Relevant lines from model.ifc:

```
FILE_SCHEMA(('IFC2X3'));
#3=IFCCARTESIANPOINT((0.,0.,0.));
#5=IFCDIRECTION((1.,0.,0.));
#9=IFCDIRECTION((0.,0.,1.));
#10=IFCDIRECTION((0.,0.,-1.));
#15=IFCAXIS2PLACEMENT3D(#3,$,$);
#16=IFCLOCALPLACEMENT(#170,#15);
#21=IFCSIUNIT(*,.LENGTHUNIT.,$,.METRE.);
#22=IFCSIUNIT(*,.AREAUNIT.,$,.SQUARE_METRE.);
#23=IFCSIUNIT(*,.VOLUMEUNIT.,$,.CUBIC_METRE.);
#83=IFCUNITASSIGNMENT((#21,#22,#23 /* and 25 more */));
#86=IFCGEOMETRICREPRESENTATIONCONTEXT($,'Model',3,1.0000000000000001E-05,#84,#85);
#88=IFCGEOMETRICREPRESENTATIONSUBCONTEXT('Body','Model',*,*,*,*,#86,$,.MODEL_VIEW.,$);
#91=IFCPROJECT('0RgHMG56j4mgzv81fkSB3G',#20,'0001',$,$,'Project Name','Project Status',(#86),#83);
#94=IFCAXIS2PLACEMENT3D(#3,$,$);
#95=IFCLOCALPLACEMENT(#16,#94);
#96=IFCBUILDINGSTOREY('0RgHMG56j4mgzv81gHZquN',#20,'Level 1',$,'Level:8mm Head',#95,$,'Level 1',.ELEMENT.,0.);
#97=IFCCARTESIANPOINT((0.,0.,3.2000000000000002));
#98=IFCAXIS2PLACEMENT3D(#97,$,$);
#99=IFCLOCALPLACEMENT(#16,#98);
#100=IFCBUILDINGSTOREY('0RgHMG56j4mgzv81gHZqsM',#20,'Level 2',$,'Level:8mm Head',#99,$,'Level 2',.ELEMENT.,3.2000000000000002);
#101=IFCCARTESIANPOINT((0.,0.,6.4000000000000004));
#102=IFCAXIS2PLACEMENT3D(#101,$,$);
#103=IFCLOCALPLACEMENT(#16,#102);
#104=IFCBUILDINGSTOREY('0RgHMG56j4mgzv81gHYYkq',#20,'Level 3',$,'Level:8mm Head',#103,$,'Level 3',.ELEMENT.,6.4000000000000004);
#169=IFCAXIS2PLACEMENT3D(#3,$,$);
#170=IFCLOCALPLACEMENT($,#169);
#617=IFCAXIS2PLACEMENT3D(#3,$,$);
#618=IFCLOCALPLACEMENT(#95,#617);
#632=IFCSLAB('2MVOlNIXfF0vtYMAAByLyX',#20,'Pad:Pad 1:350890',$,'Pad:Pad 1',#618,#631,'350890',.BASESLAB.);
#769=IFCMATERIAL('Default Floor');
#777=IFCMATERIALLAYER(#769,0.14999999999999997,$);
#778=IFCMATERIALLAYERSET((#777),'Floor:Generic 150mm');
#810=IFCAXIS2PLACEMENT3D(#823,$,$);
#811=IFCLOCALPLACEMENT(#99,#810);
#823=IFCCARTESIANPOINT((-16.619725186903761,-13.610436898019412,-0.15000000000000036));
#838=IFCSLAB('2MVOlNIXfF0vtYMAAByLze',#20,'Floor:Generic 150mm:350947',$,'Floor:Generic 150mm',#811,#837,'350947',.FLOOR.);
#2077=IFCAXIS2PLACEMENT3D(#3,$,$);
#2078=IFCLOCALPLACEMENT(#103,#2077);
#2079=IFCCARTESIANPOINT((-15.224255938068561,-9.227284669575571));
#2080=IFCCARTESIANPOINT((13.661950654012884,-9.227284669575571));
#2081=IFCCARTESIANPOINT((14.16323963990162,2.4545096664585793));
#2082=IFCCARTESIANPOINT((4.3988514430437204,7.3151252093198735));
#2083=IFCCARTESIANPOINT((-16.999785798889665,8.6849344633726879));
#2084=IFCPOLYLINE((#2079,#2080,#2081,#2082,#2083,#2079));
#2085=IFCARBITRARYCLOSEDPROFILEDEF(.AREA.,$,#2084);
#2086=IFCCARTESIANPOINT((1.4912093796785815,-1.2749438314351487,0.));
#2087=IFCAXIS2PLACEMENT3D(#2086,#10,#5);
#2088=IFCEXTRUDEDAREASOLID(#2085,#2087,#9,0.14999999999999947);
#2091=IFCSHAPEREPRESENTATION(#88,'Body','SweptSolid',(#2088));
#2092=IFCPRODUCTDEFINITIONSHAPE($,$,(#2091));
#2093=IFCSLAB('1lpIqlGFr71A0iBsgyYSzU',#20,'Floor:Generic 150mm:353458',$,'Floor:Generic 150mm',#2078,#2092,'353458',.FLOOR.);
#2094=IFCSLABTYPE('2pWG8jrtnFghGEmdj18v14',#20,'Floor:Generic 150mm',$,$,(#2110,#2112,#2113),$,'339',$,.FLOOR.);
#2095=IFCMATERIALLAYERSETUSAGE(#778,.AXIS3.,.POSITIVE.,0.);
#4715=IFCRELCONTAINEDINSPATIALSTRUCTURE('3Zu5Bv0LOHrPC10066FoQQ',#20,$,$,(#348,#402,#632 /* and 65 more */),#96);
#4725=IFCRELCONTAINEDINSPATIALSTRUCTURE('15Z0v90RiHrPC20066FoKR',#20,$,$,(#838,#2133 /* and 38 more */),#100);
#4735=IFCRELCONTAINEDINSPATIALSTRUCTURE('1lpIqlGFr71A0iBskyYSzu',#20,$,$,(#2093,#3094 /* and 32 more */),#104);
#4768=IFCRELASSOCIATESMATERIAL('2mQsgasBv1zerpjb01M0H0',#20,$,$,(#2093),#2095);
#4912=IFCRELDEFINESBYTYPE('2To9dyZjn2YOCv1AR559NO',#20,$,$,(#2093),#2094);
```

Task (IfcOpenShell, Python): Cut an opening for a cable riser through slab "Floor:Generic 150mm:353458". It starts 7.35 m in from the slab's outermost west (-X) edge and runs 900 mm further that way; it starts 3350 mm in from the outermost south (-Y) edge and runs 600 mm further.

```python
import numpy as np
import ifcopenshell
import ifcopenshell.api.feature
import ifcopenshell.api.geometry
import ifcopenshell.api.root
import ifcopenshell.geom
import ifcopenshell.util.placement
import ifcopenshell.util.representation
import ifcopenshell.util.shape
import ifcopenshell.util.unit

model = ifcopenshell.open("model.ifc")
unit_scale = ifcopenshell.util.unit.calculate_unit_scale(model)
settings = ifcopenshell.geom.settings()


def volume(element):
    """Net volume in cubic metres, openings subtracted."""
    shape = ifcopenshell.geom.create_shape(settings, element)
    return ifcopenshell.util.shape.get_volume(shape.geometry)


slab = model.by_guid("1lpIqlGFr71A0iBsgyYSzU")
before = volume(slab)

# Extent in the slab's own axes, in metres. The edges named are its -X and -Y sides.
slab_shape = ifcopenshell.geom.create_shape(settings, slab)
vertices = ifcopenshell.util.shape.get_vertices(slab_shape.geometry)
x_min, y_min, bottom = vertices.min(axis=0)
top = vertices[:, 2].max()

opening = ifcopenshell.api.root.create_entity(model, ifc_class="IfcOpeningElement", name="Cable riser opening")
context = ifcopenshell.util.representation.get_context(model, "Model", "Body", "MODEL_VIEW")
width, depth = 0.9, 0.6
outline = [(0.0, 0.0), (width, 0.0), (width, depth), (0.0, depth), (0.0, 0.0)]
# Overshoot both faces by 50 mm so the cut is clean.
shape = ifcopenshell.api.geometry.add_slab_representation(
    model, context=context, depth=top - bottom + 0.1, polyline=outline
)
ifcopenshell.api.geometry.assign_representation(model, product=opening, representation=shape)

matrix = ifcopenshell.util.placement.get_local_placement(slab.ObjectPlacement)
matrix[:, 3] = matrix @ np.append(np.array([x_min + 7.35, y_min + 3.35, bottom - 0.05]) / unit_scale, 1.0)
ifcopenshell.api.geometry.edit_object_placement(model, product=opening, matrix=matrix, is_si=False)
ifcopenshell.api.feature.add_feature(model, feature=opening, element=slab)

after = volume(slab)

print(f"slab volume {before:.3f} -> {after:.3f} m3")

model.write("model_edited.ifc")
```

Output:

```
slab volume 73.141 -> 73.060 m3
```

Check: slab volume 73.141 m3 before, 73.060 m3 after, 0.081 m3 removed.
